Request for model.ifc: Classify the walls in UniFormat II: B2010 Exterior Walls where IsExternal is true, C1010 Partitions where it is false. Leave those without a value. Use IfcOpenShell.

First a look at what the model holds.

```python
import ifcopenshell
import ifcopenshell.util.element

model = ifcopenshell.open("model.ifc")
print(model.schema)
print("classifications:", [c.Name for c in model.by_type("IfcClassification")])
values = [ifcopenshell.util.element.get_pset(e, "Pset_WallCommon", "IsExternal") for e in model.by_type("IfcWall")]
for value in (True, False, None):
    print("IsExternal", value, values.count(value))
```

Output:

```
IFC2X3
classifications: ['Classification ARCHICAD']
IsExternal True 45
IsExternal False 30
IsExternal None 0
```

```python
import ifcopenshell
import ifcopenshell.api.classification
import ifcopenshell.util.element

model = ifcopenshell.open("model.ifc")

# IFC2X3 requires Source and Edition and has no link from the project to the system.
system = model.create_entity("IfcClassification", Source="ASTM", Edition="E1557", Name="UniFormat II")

walls = model.by_type("IfcWall")
external = {e: ifcopenshell.util.element.get_pset(e, "Pset_WallCommon", "IsExternal") for e in walls}
for flag, code, name in ((True, "B2010", "Exterior Walls"), (False, "C1010", "Partitions")):
    products = [e for e in walls if external[e] is flag]
    ifcopenshell.api.classification.add_reference(
        model, products=products, classification=system, identification=code, name=name
    )
    print(code, len(products))

model.write("model_v2.ifc")
```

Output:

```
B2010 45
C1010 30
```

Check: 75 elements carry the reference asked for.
